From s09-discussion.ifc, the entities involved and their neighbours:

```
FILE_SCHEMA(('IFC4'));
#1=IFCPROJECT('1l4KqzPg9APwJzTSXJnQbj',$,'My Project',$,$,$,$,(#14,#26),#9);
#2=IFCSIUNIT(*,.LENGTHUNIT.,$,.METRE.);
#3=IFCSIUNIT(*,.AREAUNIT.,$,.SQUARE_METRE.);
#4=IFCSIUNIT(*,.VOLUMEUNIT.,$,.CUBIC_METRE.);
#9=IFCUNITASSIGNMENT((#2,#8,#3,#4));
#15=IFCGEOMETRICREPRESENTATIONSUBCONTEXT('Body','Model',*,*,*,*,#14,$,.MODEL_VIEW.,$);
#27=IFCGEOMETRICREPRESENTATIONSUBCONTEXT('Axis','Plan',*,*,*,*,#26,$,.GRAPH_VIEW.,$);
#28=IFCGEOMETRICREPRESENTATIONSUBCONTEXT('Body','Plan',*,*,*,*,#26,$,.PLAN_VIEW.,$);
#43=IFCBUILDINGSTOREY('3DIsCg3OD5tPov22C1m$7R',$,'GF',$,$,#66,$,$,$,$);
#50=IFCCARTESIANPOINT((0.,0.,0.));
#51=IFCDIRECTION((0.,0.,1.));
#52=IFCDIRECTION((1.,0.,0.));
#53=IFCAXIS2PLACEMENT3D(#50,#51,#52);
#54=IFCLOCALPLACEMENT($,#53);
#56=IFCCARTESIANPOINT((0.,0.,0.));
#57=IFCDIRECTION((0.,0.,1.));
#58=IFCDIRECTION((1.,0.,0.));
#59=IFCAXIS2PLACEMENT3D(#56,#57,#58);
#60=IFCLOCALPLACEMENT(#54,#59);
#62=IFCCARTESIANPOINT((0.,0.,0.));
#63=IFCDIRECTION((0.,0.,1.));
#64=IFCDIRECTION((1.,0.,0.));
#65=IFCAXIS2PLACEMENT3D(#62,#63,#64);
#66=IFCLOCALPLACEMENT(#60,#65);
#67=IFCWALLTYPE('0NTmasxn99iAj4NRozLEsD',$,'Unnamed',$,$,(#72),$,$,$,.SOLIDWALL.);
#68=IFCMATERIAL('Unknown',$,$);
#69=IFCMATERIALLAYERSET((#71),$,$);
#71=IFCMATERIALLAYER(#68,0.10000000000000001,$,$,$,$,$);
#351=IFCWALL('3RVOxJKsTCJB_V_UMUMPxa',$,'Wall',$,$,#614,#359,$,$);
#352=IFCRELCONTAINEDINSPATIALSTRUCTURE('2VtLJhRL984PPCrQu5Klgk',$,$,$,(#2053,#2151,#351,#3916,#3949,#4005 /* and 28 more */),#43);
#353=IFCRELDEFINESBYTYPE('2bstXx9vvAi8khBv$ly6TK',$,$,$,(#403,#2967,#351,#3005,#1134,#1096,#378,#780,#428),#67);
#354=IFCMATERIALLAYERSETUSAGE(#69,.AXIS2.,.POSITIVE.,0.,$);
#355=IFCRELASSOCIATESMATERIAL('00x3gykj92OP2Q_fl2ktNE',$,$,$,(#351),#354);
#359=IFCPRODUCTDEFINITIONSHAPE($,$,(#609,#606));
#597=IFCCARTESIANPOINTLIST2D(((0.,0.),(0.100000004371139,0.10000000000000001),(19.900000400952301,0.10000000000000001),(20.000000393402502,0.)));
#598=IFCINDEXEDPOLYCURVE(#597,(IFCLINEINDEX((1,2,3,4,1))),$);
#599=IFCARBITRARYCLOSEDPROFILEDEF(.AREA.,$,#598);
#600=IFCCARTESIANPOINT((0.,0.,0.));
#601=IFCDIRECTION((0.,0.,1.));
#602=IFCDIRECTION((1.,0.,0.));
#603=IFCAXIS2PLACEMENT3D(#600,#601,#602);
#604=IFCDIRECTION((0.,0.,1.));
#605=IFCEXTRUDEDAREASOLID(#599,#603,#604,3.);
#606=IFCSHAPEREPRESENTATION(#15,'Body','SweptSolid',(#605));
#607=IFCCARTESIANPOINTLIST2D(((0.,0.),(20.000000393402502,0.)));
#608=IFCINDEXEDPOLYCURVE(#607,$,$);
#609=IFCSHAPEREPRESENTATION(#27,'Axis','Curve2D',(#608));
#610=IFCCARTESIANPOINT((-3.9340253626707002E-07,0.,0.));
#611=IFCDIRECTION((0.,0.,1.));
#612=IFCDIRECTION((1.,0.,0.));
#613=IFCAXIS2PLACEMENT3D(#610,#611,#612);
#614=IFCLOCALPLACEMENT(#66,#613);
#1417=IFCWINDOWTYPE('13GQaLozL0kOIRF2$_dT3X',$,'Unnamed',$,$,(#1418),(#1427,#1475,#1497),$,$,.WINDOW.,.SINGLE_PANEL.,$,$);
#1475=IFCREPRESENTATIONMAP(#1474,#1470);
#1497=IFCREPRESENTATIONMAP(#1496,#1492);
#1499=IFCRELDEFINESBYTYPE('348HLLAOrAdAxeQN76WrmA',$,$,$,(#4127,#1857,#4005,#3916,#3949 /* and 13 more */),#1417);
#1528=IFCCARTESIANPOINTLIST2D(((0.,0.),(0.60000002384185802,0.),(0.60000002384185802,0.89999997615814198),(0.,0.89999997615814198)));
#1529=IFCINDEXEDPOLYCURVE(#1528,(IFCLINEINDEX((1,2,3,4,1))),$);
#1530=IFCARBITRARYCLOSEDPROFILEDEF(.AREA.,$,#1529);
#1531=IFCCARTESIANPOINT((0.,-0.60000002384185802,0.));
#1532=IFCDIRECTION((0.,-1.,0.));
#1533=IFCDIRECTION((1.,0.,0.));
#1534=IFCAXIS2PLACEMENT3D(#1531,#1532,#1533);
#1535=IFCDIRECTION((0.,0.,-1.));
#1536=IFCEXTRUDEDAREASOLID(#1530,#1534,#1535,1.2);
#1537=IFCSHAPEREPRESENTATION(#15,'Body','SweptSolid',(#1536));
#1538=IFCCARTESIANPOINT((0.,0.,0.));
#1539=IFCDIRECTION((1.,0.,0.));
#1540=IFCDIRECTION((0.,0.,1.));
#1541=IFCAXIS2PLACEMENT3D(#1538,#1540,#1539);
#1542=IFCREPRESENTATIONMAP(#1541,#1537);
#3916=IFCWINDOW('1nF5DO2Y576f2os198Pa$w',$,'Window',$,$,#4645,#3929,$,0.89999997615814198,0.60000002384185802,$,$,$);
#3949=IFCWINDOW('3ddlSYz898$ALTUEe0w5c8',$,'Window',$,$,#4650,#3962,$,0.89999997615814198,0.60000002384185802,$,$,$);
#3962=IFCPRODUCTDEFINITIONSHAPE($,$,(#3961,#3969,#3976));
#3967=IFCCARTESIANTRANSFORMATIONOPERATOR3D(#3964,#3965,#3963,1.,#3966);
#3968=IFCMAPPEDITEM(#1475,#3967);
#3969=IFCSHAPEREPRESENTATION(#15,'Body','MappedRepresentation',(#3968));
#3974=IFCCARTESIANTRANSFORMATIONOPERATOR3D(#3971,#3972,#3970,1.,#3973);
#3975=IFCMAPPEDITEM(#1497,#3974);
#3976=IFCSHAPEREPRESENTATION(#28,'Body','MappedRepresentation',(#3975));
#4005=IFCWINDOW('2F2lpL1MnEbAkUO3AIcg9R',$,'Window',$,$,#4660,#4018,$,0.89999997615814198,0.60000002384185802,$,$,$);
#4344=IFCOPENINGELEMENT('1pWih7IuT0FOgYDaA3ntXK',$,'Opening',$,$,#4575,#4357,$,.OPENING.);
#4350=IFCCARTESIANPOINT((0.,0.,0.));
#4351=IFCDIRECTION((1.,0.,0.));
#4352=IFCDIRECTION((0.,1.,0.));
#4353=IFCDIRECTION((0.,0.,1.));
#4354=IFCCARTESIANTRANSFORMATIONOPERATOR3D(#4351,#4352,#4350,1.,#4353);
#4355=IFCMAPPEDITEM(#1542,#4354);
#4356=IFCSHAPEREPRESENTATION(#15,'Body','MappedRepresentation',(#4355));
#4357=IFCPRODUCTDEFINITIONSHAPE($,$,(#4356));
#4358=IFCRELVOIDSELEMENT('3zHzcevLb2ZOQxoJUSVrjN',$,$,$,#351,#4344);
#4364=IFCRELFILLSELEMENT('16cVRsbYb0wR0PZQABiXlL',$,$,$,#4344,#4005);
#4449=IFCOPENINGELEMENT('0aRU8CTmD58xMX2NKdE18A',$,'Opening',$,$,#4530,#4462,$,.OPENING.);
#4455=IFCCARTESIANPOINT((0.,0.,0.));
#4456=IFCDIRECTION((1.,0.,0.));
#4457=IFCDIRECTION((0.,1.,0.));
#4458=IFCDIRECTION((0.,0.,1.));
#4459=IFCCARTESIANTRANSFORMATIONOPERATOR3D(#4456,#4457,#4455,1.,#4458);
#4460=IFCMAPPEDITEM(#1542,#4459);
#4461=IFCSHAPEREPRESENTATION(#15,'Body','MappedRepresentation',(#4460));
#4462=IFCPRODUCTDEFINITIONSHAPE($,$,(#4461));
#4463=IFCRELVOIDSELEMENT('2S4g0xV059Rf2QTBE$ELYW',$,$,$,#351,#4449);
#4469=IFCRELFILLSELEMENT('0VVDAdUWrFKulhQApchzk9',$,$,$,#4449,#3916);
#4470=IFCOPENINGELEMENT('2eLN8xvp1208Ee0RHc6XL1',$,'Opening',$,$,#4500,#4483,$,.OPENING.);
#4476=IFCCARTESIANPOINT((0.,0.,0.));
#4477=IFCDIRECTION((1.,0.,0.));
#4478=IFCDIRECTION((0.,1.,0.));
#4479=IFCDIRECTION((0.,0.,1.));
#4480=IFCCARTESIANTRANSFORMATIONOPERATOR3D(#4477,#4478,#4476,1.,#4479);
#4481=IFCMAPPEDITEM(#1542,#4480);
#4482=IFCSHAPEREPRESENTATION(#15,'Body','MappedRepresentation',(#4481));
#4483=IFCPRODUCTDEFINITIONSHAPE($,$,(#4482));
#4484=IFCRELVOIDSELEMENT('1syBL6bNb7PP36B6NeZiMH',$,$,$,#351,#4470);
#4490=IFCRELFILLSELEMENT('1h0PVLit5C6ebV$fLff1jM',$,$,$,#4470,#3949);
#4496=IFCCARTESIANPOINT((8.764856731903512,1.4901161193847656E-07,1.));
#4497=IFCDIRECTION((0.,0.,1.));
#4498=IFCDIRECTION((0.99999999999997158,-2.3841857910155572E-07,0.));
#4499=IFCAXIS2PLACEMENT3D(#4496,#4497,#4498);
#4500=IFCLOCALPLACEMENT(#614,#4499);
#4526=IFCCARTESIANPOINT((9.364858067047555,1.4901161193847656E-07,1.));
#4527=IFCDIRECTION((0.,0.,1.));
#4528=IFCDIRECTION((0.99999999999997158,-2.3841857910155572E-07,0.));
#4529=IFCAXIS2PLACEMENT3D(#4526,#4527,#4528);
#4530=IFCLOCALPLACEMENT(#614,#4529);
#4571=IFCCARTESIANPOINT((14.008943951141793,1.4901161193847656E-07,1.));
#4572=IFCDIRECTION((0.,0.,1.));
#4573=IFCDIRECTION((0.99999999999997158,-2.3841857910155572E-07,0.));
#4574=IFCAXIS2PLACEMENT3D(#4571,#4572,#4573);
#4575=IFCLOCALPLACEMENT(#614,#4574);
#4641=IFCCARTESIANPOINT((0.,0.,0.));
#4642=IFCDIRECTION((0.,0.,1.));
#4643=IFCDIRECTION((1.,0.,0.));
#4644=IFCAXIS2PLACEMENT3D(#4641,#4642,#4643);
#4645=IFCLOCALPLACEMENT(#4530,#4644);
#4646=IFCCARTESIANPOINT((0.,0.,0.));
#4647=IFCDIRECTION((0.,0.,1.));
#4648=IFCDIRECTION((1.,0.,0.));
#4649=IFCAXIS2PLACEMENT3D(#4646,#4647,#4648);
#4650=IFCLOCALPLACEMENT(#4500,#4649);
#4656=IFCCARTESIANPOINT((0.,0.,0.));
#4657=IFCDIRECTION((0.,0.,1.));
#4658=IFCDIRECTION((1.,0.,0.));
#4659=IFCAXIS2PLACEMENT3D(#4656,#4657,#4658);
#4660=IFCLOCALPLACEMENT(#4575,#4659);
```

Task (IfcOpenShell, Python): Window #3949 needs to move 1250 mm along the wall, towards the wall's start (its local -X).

```python
import ifcopenshell
import ifcopenshell.api.geometry
import ifcopenshell.util.placement
import ifcopenshell.util.unit

model = ifcopenshell.open("s09-discussion.ifc")
unit_scale = ifcopenshell.util.unit.calculate_unit_scale(model)

window = model.by_guid("3ddlSYz898$ALTUEe0w5c8")
opening = window.FillsVoids[0].RelatingOpeningElement
wall = opening.VoidsElements[0].RelatingBuildingElement

wall_matrix = ifcopenshell.util.placement.get_local_placement(wall.ObjectPlacement)
shift = wall_matrix[:3, 0] * -1.25 / unit_scale
before = ifcopenshell.util.placement.get_local_placement(window.ObjectPlacement)[:3, 3].copy()

# The window is placed relative to its opening, so it follows when the opening moves.
matrix = ifcopenshell.util.placement.get_local_placement(opening.ObjectPlacement)
matrix[:3, 3] += shift
ifcopenshell.api.geometry.edit_object_placement(
    model, product=opening, matrix=matrix, is_si=False, should_transform_children=True
)

after = ifcopenshell.util.placement.get_local_placement(window.ObjectPlacement)[:3, 3]
print("window moved by", (after - before).round(3) + 0.0)

model.write("s09-discussion_edited.ifc")
```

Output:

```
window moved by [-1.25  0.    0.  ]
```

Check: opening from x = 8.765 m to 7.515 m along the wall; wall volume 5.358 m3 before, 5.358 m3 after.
